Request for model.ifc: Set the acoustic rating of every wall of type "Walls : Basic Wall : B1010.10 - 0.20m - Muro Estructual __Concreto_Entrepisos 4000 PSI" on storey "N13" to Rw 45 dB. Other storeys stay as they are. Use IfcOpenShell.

First a look at what the model holds.

```python
import ifcopenshell
import ifcopenshell.util.element

model = ifcopenshell.open("model.ifc")
print(model.schema)
storey = next(s for s in model.by_type("IfcBuildingStorey") if s.Name == "N13")
walls = [e for e in ifcopenshell.util.element.get_decomposition(storey) if e.is_a("IfcWall")]
seen = {}
for e in walls:
    element_type = ifcopenshell.util.element.get_type(e)
    key = (element_type.Name if element_type != e and element_type else None, ifcopenshell.util.element.get_pset(e, "Pset_WallCommon", "AcousticRating"))
    seen[key] = seen.get(key, 0) + 1
for (name, value), count in sorted(seen.items(), key=str):
    print(count, "x", name, "|", value)
```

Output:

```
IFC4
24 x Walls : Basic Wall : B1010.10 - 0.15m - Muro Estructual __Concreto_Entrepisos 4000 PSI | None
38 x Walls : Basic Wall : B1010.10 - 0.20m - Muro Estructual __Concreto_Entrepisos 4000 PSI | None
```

```python
import ifcopenshell
import ifcopenshell.api.pset
import ifcopenshell.util.element

model = ifcopenshell.open("model.ifc")

storey = next(s for s in model.by_type("IfcBuildingStorey") if s.Name == "N13")
walls = [e for e in ifcopenshell.util.element.get_decomposition(storey) if e.is_a("IfcWall")]

count = 0
for e in walls:
    element_type = ifcopenshell.util.element.get_type(e)
    if element_type in (None, e) or element_type.Name != "Walls : Basic Wall : B1010.10 - 0.20m - Muro Estructual __Concreto_Entrepisos 4000 PSI":
        continue
    # add_pset returns the element's existing set when there is one.
    pset = ifcopenshell.api.pset.add_pset(model, product=e, name="Pset_WallCommon")
    ifcopenshell.api.pset.edit_pset(model, pset=pset, properties={"AcousticRating": "Rw 45 dB"})
    count += 1

print(count, "walls updated")

model.write("model_v2.ifc")
```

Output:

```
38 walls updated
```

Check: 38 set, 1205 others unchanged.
